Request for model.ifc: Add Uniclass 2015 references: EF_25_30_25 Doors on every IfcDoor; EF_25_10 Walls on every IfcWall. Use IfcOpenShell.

First a look at what the model holds.

```python
import ifcopenshell

model = ifcopenshell.open("model.ifc")
print(model.schema)
print("classifications:", [c.Name for c in model.by_type("IfcClassification")])
for ifc_class in ("IfcDoor", "IfcRoof", "IfcStair", "IfcWall", "IfcWindow"):
    print(ifc_class, len(model.by_type(ifc_class)))
```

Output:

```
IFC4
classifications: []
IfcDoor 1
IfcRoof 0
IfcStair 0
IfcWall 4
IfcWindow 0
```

```python
import ifcopenshell
import ifcopenshell.api.classification

model = ifcopenshell.open("model.ifc")

system = ifcopenshell.api.classification.add_classification(model, classification="Uniclass 2015")

codes = {
    "IfcDoor": ("EF_25_30_25", "Doors"),
    "IfcWall": ("EF_25_10", "Walls"),
}
for ifc_class, (code, name) in codes.items():
    products = model.by_type(ifc_class)
    ifcopenshell.api.classification.add_reference(
        model, products=products, classification=system, identification=code, name=name
    )
    print(code, len(products))

model.write("model-out.ifc")
```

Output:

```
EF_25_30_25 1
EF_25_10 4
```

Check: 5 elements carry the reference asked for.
